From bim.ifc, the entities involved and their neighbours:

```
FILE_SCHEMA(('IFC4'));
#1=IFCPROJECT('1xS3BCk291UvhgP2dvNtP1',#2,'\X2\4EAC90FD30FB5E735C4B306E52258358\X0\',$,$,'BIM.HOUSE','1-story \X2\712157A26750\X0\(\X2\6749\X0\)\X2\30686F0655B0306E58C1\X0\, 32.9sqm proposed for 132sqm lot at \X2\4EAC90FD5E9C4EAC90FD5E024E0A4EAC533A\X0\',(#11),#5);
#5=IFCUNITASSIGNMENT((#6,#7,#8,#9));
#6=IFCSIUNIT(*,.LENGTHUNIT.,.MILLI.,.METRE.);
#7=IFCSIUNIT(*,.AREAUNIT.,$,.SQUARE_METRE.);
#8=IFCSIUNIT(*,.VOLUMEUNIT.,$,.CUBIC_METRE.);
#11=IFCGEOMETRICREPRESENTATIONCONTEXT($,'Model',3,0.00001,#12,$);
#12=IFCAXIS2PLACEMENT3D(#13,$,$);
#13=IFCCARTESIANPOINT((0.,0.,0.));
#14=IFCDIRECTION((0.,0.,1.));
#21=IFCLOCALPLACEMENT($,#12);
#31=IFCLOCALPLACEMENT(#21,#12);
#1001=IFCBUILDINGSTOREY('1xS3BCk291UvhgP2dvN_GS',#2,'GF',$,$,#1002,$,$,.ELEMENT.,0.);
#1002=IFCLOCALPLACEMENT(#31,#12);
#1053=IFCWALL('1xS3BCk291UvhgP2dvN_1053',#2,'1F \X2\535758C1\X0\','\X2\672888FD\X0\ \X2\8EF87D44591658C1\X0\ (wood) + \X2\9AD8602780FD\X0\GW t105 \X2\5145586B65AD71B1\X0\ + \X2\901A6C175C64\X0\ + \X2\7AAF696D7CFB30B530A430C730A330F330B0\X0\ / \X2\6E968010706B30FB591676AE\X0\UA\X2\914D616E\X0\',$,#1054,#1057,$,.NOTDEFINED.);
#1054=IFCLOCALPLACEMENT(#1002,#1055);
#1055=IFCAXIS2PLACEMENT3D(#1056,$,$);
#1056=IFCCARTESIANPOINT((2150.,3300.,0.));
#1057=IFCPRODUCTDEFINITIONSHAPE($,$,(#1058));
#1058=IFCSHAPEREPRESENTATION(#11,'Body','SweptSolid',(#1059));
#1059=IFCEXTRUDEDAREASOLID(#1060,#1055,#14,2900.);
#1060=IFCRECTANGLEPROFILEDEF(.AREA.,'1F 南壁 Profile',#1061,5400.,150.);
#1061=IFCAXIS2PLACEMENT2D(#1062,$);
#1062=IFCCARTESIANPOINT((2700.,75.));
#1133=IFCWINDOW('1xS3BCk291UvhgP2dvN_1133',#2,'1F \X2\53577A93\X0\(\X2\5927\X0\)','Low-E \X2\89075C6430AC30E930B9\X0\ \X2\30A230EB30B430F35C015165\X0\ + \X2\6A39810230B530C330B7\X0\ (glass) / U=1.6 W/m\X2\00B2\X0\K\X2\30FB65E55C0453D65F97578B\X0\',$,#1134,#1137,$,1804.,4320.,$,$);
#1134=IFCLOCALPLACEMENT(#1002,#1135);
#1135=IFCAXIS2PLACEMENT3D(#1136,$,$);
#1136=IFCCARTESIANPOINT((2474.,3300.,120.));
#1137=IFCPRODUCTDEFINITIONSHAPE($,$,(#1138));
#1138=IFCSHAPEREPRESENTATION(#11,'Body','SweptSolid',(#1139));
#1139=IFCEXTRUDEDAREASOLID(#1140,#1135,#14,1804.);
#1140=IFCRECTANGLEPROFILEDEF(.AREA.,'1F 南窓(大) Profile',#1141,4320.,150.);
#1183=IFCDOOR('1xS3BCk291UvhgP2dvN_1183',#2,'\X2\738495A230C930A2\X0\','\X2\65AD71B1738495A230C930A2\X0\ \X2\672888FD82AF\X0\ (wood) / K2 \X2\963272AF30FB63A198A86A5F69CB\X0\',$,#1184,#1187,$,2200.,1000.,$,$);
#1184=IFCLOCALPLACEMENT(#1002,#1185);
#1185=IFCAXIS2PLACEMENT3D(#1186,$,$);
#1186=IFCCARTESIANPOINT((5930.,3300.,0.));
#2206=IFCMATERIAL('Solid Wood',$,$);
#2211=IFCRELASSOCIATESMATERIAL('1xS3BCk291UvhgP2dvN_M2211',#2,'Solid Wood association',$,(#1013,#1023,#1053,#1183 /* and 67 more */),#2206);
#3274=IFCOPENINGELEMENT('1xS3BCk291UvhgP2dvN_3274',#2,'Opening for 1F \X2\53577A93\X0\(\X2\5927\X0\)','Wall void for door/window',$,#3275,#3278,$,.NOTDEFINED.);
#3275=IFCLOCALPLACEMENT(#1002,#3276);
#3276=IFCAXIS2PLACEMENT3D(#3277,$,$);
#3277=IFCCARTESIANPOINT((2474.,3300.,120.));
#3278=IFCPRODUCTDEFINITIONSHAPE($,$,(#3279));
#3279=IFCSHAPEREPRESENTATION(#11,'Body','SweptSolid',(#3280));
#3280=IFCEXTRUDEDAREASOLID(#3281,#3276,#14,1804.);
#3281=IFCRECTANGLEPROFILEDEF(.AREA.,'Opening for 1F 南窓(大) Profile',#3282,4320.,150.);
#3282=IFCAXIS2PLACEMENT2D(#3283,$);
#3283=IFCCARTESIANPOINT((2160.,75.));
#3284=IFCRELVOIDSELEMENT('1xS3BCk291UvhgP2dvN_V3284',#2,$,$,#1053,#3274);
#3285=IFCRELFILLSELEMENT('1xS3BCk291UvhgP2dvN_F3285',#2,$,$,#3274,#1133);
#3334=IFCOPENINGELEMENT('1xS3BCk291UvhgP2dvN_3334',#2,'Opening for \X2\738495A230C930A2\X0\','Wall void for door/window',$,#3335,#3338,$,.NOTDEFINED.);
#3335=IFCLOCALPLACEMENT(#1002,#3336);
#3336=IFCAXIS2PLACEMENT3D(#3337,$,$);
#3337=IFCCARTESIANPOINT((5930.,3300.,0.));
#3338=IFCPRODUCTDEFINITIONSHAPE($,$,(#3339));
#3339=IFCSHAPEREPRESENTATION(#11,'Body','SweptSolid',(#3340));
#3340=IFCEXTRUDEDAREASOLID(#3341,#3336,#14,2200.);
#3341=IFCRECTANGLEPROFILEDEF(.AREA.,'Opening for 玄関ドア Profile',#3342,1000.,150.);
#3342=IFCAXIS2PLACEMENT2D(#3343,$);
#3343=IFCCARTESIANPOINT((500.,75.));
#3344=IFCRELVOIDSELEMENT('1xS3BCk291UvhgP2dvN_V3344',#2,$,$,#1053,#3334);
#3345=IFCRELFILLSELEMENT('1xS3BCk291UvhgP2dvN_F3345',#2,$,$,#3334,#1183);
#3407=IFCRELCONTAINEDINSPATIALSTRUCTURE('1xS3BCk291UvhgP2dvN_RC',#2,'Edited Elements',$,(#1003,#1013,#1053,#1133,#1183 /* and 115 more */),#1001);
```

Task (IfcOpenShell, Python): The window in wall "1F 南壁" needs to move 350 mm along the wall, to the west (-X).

```python
import ifcopenshell
import ifcopenshell.api.geometry
import ifcopenshell.util.placement
import ifcopenshell.util.unit

model = ifcopenshell.open("bim.ifc")
unit_scale = ifcopenshell.util.unit.calculate_unit_scale(model)

window = model.by_id(1133)
opening = window.FillsVoids[0].RelatingOpeningElement
wall = opening.VoidsElements[0].RelatingBuildingElement

wall_matrix = ifcopenshell.util.placement.get_local_placement(wall.ObjectPlacement)
shift = wall_matrix[:3, 0] * -0.35 / unit_scale
before = ifcopenshell.util.placement.get_local_placement(window.ObjectPlacement)[:3, 3].copy()

# The window is not placed relative to its opening, so move both.
for product in (opening, window):
    matrix = ifcopenshell.util.placement.get_local_placement(product.ObjectPlacement)
    matrix[:3, 3] += shift
    ifcopenshell.api.geometry.edit_object_placement(model, product=product, matrix=matrix, is_si=False)

after = ifcopenshell.util.placement.get_local_placement(window.ObjectPlacement)[:3, 3]
print("window moved by", (after - before).round(3) + 0.0)

model.write("bim-out.ifc")
```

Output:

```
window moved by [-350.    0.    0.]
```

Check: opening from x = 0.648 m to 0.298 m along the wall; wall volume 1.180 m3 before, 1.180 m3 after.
